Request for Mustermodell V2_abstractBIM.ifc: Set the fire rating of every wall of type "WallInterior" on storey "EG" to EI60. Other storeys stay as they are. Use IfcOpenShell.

First a look at what the model holds.

```python
import ifcopenshell
import ifcopenshell.util.element

model = ifcopenshell.open("Mustermodell V2_abstractBIM.ifc")
print(model.schema)
storey = next(s for s in model.by_type("IfcBuildingStorey") if s.Name == "EG")
walls = [e for e in ifcopenshell.util.element.get_decomposition(storey) if e.is_a("IfcWall")]
seen = {}
for e in walls:
    element_type = ifcopenshell.util.element.get_type(e)
    key = (element_type.Name if element_type != e and element_type else None, ifcopenshell.util.element.get_pset(e, "Pset_WallCommon", "FireRating"))
    seen[key] = seen.get(key, 0) + 1
for (name, value), count in sorted(seen.items(), key=str):
    print(count, "x", name, "|", value)
```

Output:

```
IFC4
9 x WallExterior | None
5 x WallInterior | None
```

```python
import ifcopenshell
import ifcopenshell.api.pset
import ifcopenshell.util.element

model = ifcopenshell.open("Mustermodell V2_abstractBIM.ifc")

storey = next(s for s in model.by_type("IfcBuildingStorey") if s.Name == "EG")
walls = [e for e in ifcopenshell.util.element.get_decomposition(storey) if e.is_a("IfcWall")]

count = 0
for e in walls:
    element_type = ifcopenshell.util.element.get_type(e)
    if element_type in (None, e) or element_type.Name != "WallInterior":
        continue
    # add_pset returns the element's existing set when there is one.
    pset = ifcopenshell.api.pset.add_pset(model, product=e, name="Pset_WallCommon")
    ifcopenshell.api.pset.edit_pset(model, pset=pset, properties={"FireRating": "EI60"})
    count += 1

print(count, "walls updated")

model.write("Mustermodell V2_abstractBIM_rev.ifc")
```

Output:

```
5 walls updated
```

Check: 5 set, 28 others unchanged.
